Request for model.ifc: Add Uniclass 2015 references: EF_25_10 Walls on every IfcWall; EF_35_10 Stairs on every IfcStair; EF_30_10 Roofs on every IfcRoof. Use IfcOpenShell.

First a look at what the model holds.

```python
import ifcopenshell

model = ifcopenshell.open("model.ifc")
print(model.schema)
print("classifications:", [c.Name for c in model.by_type("IfcClassification")])
for ifc_class in ("IfcDoor", "IfcRoof", "IfcStair", "IfcWall", "IfcWindow"):
    print(ifc_class, len(model.by_type(ifc_class)))
```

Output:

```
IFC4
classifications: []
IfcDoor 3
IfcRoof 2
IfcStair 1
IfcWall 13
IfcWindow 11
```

```python
import ifcopenshell
import ifcopenshell.api.classification

model = ifcopenshell.open("model.ifc")

system = ifcopenshell.api.classification.add_classification(model, classification="Uniclass 2015")

codes = {
    "IfcWall": ("EF_25_10", "Walls"),
    "IfcStair": ("EF_35_10", "Stairs"),
    "IfcRoof": ("EF_30_10", "Roofs"),
}
for ifc_class, (code, name) in codes.items():
    products = model.by_type(ifc_class)
    ifcopenshell.api.classification.add_reference(
        model, products=products, classification=system, identification=code, name=name
    )
    print(code, len(products))

model.write("model_v2.ifc")
```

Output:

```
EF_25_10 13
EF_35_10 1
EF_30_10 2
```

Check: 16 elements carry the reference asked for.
